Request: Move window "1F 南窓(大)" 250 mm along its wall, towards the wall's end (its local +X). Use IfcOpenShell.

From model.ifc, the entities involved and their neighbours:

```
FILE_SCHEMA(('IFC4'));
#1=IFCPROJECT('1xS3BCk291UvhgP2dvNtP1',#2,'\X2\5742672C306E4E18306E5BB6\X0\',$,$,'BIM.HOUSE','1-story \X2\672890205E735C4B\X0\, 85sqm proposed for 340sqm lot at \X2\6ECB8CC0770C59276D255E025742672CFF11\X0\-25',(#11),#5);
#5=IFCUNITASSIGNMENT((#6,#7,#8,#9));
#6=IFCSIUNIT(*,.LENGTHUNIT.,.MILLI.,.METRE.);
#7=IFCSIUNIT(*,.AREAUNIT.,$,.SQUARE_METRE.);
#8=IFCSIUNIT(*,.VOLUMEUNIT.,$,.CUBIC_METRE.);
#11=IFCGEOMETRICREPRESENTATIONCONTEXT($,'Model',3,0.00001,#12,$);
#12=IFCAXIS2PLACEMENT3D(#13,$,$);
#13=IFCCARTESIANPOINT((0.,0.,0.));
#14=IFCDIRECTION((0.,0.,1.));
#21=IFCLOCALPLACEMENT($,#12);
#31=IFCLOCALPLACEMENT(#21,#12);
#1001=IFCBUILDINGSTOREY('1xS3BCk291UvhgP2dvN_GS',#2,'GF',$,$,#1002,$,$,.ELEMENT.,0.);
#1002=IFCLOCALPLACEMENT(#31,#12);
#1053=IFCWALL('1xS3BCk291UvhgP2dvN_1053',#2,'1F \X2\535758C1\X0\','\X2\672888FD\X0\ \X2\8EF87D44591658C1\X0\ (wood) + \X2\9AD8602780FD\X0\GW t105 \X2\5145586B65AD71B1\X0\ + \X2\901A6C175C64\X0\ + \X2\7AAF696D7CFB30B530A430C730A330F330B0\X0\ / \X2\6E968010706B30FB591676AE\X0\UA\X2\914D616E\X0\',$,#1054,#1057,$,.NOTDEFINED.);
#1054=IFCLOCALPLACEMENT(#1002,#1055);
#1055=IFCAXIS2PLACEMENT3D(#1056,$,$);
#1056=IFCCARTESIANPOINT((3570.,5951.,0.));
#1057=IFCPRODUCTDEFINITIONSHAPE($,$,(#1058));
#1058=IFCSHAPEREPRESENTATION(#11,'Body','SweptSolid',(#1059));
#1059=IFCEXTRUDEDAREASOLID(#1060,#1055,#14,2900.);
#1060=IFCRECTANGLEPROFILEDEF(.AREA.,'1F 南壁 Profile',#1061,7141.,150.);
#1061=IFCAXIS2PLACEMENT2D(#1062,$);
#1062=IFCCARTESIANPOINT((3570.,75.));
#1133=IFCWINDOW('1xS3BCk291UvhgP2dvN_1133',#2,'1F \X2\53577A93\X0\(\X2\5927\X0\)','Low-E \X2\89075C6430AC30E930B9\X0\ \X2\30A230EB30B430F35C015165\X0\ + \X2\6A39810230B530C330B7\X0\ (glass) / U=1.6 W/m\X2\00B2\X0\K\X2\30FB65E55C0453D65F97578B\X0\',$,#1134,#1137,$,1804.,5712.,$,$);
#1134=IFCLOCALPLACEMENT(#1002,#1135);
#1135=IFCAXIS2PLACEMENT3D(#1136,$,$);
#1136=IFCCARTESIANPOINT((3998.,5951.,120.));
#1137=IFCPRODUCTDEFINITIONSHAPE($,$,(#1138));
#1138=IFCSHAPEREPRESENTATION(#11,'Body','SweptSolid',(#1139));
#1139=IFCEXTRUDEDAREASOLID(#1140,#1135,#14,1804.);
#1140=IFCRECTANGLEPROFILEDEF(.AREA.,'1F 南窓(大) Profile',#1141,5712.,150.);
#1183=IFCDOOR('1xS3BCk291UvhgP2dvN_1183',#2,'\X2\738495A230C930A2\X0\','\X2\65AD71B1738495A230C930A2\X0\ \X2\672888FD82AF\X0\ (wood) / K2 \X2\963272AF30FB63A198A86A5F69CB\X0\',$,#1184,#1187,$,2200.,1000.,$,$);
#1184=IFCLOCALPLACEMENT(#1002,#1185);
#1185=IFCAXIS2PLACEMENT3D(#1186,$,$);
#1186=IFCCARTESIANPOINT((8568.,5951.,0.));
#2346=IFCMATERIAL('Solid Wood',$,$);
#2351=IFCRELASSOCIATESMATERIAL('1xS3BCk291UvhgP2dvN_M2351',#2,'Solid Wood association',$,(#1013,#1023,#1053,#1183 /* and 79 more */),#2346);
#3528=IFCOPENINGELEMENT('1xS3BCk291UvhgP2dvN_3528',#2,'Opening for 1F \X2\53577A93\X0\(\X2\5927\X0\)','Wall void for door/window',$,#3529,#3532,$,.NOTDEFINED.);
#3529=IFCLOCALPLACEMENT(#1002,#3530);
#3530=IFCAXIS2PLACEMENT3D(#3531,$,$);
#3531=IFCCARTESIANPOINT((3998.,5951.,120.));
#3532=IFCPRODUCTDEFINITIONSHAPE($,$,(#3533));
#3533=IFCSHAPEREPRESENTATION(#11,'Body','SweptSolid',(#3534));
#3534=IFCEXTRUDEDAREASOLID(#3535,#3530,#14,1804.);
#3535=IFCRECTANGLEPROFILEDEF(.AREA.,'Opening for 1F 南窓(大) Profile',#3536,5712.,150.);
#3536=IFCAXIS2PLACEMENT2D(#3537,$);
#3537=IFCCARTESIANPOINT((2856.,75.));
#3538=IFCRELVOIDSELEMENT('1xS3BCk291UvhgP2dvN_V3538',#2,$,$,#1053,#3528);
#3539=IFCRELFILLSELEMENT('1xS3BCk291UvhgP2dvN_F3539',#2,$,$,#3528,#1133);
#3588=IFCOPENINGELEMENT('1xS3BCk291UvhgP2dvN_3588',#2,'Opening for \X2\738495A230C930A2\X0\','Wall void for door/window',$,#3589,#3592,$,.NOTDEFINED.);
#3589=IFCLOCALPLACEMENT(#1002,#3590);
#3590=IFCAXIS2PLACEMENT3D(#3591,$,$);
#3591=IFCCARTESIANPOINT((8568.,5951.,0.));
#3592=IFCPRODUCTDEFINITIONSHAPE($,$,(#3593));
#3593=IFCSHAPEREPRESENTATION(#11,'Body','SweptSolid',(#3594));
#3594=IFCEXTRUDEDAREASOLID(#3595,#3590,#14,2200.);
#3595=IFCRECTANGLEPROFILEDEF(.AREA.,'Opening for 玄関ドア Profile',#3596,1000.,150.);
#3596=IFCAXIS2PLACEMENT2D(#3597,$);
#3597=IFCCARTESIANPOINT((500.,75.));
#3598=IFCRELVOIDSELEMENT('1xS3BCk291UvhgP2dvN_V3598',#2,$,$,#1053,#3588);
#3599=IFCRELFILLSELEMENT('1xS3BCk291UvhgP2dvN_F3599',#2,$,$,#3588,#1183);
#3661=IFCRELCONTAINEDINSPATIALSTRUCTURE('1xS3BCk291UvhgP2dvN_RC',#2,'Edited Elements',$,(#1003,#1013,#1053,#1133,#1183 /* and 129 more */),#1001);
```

```python
import ifcopenshell
import ifcopenshell.api.geometry
import ifcopenshell.util.placement

model = ifcopenshell.open("model.ifc")

window = model.by_guid("1xS3BCk291UvhgP2dvN_1133")
opening = window.FillsVoids[0].RelatingOpeningElement
wall = opening.VoidsElements[0].RelatingBuildingElement

wall_matrix = ifcopenshell.util.placement.get_local_placement(wall.ObjectPlacement)
shift = wall_matrix[:3, 0] * 250.0
before = ifcopenshell.util.placement.get_local_placement(window.ObjectPlacement)[:3, 3].copy()

# The window is not placed relative to its opening, so move both.
for product in (opening, window):
    matrix = ifcopenshell.util.placement.get_local_placement(product.ObjectPlacement)
    matrix[:3, 3] += shift
    ifcopenshell.api.geometry.edit_object_placement(model, product=product, matrix=matrix, is_si=False)

after = ifcopenshell.util.placement.get_local_placement(window.ObjectPlacement)[:3, 3]
print("window moved by", (after - before).round(3) + 0.0)

model.write("model-out.ifc")
```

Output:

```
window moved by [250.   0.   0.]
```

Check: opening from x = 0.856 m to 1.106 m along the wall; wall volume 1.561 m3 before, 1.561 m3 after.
